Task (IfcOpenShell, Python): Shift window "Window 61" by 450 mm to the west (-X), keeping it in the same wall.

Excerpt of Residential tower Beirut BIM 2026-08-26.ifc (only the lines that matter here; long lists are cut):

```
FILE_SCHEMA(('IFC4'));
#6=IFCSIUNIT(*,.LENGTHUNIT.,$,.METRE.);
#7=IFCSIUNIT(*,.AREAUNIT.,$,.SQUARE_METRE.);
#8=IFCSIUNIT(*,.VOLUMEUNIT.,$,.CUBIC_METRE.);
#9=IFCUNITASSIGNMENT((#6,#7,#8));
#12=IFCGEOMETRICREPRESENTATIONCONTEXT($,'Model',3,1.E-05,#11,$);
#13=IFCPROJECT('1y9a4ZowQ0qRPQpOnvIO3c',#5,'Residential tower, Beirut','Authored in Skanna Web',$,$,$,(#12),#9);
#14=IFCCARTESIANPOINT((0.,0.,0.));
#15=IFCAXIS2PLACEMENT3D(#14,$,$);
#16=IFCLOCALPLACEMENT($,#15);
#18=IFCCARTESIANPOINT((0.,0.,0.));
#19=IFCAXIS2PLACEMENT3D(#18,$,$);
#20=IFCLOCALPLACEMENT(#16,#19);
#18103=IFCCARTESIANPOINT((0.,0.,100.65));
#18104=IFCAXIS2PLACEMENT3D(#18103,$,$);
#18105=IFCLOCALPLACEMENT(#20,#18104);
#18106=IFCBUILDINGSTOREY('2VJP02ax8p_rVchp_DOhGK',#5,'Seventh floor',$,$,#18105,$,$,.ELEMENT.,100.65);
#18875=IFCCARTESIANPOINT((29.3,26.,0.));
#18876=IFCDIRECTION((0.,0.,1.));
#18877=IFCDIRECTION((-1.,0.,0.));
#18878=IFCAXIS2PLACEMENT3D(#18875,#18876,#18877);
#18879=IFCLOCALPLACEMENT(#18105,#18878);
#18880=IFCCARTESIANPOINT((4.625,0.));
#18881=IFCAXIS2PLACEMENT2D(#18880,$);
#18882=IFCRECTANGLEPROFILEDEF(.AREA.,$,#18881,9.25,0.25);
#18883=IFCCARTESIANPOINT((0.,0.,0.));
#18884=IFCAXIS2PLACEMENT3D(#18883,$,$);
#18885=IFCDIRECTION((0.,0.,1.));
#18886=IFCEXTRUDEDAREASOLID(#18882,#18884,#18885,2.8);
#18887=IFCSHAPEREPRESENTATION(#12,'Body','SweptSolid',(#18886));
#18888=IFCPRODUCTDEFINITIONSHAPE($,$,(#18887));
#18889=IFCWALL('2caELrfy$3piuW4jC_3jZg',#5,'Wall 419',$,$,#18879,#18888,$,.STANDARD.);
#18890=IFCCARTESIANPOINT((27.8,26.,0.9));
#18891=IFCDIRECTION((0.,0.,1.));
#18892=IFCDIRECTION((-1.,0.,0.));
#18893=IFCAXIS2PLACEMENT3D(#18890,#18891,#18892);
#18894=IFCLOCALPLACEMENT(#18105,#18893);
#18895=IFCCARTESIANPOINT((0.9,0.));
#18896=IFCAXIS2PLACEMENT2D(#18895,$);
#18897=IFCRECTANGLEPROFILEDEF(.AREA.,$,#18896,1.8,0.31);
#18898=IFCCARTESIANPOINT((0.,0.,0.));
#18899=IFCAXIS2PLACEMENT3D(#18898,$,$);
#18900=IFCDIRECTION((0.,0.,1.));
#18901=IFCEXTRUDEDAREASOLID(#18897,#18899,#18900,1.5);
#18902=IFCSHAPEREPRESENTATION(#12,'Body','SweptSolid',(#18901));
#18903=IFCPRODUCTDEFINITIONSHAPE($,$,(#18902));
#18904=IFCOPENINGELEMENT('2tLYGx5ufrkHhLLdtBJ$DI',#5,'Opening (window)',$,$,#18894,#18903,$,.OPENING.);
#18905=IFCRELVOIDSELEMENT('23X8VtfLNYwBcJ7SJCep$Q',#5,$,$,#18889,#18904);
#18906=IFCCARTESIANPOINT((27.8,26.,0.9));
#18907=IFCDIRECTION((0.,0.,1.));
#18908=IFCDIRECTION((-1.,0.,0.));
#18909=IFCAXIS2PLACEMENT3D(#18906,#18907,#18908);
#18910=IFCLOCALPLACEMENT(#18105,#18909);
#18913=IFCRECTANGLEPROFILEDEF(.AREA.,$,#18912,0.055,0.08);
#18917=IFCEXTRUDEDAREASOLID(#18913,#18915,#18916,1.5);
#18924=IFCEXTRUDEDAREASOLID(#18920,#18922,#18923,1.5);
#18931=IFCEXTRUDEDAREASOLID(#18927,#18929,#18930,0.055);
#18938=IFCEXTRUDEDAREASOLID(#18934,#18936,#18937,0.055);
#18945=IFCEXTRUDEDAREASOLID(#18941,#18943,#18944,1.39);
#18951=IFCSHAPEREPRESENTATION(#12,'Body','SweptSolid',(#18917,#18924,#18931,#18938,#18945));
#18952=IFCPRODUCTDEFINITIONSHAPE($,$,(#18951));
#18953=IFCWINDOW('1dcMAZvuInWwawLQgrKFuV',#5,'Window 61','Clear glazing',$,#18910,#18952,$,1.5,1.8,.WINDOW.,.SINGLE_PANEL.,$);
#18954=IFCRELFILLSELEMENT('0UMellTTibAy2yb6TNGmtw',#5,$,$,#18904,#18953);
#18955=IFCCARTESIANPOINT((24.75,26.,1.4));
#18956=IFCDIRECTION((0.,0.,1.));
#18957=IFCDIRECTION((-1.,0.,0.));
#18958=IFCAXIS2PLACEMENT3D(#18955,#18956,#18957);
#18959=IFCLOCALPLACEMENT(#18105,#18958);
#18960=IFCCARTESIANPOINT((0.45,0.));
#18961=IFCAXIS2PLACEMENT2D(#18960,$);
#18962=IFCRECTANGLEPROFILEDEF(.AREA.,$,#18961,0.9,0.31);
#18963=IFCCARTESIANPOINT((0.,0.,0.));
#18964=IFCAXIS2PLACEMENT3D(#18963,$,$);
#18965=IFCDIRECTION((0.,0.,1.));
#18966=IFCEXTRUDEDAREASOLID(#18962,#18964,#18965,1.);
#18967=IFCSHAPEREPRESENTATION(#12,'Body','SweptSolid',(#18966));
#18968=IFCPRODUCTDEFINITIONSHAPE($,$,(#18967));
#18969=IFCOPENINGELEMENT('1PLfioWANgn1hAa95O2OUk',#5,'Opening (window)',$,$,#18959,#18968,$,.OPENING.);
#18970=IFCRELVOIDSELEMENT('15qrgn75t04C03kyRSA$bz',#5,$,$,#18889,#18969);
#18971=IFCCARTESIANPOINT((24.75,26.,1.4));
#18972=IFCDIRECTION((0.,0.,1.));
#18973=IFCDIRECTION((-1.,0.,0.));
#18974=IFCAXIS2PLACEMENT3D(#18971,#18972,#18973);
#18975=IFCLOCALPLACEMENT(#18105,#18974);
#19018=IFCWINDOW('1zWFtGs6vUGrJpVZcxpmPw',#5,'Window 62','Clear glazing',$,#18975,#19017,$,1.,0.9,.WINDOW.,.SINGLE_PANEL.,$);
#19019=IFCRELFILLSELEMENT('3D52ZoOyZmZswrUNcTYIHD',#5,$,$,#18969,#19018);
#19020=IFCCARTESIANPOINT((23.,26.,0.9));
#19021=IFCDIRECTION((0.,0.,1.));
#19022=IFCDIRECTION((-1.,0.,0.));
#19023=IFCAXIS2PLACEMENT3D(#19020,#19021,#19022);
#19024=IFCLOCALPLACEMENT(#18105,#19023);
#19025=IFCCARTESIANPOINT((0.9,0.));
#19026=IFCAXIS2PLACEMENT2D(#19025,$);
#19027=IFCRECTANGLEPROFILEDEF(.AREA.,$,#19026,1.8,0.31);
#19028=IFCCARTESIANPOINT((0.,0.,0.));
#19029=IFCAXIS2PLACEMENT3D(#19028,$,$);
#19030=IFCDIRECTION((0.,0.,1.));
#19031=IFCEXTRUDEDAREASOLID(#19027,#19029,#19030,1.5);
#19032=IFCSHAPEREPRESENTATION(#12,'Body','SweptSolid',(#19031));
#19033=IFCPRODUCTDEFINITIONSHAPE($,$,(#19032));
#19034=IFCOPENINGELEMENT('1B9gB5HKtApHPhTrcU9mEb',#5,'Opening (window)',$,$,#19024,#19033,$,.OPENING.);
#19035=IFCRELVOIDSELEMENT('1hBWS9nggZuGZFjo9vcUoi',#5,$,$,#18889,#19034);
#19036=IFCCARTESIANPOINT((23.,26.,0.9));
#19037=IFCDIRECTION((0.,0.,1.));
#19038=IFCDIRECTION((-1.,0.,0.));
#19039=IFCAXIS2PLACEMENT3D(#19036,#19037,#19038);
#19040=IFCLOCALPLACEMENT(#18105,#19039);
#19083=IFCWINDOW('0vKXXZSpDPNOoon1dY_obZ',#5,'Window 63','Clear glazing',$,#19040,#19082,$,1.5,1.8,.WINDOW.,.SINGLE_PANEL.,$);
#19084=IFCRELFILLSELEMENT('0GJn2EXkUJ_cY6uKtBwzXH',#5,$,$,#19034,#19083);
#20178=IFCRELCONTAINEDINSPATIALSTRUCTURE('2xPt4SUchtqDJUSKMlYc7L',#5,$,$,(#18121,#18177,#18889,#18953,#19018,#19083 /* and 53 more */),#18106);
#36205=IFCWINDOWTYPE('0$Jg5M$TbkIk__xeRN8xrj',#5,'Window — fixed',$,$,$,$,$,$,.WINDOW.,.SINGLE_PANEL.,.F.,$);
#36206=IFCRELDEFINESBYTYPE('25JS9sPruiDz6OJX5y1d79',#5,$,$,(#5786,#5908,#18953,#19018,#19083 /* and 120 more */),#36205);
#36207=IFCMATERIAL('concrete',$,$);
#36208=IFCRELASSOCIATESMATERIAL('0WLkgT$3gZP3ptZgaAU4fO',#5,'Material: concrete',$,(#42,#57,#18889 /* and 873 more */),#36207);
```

```python
import ifcopenshell
import ifcopenshell.api.geometry
import ifcopenshell.util.placement

model = ifcopenshell.open("Residential tower Beirut BIM 2026-08-26.ifc")

window = model.by_guid("1dcMAZvuInWwawLQgrKFuV")
opening = window.FillsVoids[0].RelatingOpeningElement
wall = opening.VoidsElements[0].RelatingBuildingElement

wall_matrix = ifcopenshell.util.placement.get_local_placement(wall.ObjectPlacement)
shift = wall_matrix[:3, 0] * 0.45
before = ifcopenshell.util.placement.get_local_placement(window.ObjectPlacement)[:3, 3].copy()

# The window is not placed relative to its opening, so move both.
for product in (opening, window):
    matrix = ifcopenshell.util.placement.get_local_placement(product.ObjectPlacement)
    matrix[:3, 3] += shift
    ifcopenshell.api.geometry.edit_object_placement(model, product=product, matrix=matrix, is_si=False)

after = ifcopenshell.util.placement.get_local_placement(window.ObjectPlacement)[:3, 3]
print("window moved by", (after - before).round(3) + 0.0)

model.write("Residential tower Beirut BIM 2026-08-26_updated.ifc")
```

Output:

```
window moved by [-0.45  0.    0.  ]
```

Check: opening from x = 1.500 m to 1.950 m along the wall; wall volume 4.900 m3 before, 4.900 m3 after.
